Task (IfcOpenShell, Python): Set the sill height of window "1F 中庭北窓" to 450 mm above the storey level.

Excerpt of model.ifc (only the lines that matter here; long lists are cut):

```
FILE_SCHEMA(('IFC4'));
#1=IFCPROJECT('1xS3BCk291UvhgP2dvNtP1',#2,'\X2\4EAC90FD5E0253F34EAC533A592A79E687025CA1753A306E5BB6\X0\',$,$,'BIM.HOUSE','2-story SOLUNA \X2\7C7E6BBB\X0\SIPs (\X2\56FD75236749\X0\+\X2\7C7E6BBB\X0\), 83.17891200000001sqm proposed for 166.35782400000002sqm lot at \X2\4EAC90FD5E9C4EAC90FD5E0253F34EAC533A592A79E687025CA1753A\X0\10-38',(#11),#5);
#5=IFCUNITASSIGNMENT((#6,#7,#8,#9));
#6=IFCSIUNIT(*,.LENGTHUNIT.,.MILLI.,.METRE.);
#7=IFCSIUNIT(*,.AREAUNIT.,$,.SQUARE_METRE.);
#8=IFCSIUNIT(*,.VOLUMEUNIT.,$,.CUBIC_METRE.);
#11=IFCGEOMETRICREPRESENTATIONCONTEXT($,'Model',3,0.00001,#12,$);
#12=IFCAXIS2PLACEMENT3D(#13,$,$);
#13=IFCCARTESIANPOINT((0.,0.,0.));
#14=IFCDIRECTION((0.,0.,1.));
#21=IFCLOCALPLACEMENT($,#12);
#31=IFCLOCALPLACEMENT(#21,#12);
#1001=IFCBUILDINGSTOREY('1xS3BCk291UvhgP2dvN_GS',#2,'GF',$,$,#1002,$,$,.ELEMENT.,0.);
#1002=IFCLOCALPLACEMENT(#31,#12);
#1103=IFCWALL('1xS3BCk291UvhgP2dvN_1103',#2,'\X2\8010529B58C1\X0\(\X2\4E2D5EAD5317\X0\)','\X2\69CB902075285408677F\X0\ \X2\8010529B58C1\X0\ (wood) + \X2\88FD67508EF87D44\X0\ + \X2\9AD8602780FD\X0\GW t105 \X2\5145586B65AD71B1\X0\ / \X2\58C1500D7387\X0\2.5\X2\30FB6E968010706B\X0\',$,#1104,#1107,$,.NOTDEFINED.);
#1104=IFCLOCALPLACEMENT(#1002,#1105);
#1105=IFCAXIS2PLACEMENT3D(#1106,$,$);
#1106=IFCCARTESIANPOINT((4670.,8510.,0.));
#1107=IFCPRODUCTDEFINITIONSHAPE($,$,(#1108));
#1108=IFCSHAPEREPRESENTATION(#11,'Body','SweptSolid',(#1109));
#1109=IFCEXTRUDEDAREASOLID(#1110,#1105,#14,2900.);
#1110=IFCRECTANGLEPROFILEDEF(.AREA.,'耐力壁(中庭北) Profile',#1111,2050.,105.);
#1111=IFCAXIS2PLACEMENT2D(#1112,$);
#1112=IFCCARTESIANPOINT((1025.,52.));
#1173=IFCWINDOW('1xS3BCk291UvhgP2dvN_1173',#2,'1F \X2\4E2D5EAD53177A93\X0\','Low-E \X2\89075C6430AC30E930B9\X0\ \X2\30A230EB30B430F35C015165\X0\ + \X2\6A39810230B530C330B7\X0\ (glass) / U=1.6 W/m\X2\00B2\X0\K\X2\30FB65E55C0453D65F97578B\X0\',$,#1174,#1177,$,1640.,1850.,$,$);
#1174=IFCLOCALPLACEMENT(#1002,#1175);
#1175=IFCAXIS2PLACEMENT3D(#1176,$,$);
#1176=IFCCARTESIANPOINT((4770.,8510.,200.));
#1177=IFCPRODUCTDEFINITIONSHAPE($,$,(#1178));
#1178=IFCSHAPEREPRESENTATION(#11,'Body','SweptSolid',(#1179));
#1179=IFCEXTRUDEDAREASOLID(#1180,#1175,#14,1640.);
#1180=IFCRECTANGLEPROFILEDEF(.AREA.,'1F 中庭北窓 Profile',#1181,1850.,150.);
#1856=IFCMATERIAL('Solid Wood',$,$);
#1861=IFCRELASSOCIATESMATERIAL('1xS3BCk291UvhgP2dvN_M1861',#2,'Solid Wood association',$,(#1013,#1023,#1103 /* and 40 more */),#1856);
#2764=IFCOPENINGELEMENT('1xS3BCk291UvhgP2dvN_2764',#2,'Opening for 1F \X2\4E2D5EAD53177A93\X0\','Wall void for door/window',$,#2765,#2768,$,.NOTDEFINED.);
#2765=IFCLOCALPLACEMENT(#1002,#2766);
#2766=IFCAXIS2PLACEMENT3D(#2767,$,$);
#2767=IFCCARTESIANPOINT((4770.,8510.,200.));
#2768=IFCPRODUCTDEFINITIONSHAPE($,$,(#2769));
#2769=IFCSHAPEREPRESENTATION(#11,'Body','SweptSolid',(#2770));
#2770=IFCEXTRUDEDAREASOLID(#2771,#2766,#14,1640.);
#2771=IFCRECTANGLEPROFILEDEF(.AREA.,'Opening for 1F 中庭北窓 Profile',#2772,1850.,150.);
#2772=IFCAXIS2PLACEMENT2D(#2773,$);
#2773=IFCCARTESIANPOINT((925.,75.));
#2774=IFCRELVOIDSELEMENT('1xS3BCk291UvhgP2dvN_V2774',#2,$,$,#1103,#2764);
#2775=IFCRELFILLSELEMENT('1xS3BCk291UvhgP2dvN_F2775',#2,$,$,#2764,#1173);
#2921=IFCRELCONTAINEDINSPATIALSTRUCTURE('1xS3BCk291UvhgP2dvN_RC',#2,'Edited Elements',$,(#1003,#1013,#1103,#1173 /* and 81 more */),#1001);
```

```python
import numpy as np
import ifcopenshell
import ifcopenshell.api.geometry
import ifcopenshell.geom
import ifcopenshell.util.element
import ifcopenshell.util.placement
import ifcopenshell.util.shape
import ifcopenshell.util.unit

model = ifcopenshell.open("model.ifc")
unit_scale = ifcopenshell.util.unit.calculate_unit_scale(model)

window = model.by_guid("1xS3BCk291UvhgP2dvN_1173")
opening = window.FillsVoids[0].RelatingOpeningElement
storey = ifcopenshell.util.element.get_container(window, ifc_class="IfcBuildingStorey")
level = ifcopenshell.util.placement.get_local_placement(storey.ObjectPlacement)[2, 3]

# The opening's origin need not be at the sill, so measure its lowest point.
shape = ifcopenshell.geom.create_shape(ifcopenshell.geom.settings(), opening)
bottom = ifcopenshell.util.shape.get_shape_bottom_elevation(shape, shape.geometry) / unit_scale
dz = level + 450.0 - bottom

shift = np.array([0.0, 0.0, dz])
# The window is not placed relative to its opening, so move both.
for product in (opening, window):
    matrix = ifcopenshell.util.placement.get_local_placement(product.ObjectPlacement)
    matrix[:3, 3] += shift
    ifcopenshell.api.geometry.edit_object_placement(model, product=product, matrix=matrix, is_si=False)

print(f"moved by {dz * unit_scale:+.3f} m")

model.write("model_v2.ifc")
```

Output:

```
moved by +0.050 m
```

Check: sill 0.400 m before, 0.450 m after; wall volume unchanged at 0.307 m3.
